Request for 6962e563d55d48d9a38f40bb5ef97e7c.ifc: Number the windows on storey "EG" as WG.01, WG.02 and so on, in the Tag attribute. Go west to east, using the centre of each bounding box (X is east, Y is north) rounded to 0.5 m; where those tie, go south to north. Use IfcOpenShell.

First a look at what the model holds.

```python
import ifcopenshell
import ifcopenshell.util.element
import ifcopenshell.util.placement

model = ifcopenshell.open("6962e563d55d48d9a38f40bb5ef97e7c.ifc")
print(model.schema)
storey = next(s for s in model.by_type("IfcBuildingStorey") if s.Name == "EG")
windows = [e for e in ifcopenshell.util.element.get_decomposition(storey) if e.is_a("IfcWindow")]
for e in sorted(windows, key=lambda e: e.id()):
    origin = ifcopenshell.util.placement.get_local_placement(e.ObjectPlacement)[:3, 3]
    print(e.id(), e.Tag, e.Name, origin.round(2) + 0.0, sep=" | ")
```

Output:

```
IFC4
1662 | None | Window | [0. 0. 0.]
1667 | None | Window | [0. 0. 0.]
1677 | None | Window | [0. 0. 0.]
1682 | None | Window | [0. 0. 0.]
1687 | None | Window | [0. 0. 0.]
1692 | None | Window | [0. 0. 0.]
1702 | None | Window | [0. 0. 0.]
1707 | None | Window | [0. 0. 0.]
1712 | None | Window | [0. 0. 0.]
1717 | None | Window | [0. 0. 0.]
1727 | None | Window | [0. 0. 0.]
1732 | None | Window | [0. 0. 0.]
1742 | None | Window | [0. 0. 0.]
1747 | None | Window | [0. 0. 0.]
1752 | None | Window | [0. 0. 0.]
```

```python
import ifcopenshell
import ifcopenshell.geom
import ifcopenshell.util.element
import ifcopenshell.util.shape

model = ifcopenshell.open("6962e563d55d48d9a38f40bb5ef97e7c.ifc")
settings = ifcopenshell.geom.settings()
settings.set("use-world-coords", True)


def centre(element):
    shape = ifcopenshell.geom.create_shape(settings, element)
    return ifcopenshell.util.shape.get_bbox_centroid(shape.geometry)


storey = next(s for s in model.by_type("IfcBuildingStorey") if s.Name == "EG")
windows = [e for e in ifcopenshell.util.element.get_decomposition(storey) if e.is_a("IfcWindow")]

# Insertion points can sit at a corner or the storey origin, so sort by the geometry (in metres).
centres = {e: centre(e) for e in windows}
windows.sort(key=lambda e: (round(centres[e][0] / 0.5), centres[e][1]))

for i, e in enumerate(windows, start=1):
    number = f"WG.{i:02d}"
    e.Tag = number
    print(e.id(), number)

model.write("6962e563d55d48d9a38f40bb5ef97e7c_rev.ifc")
```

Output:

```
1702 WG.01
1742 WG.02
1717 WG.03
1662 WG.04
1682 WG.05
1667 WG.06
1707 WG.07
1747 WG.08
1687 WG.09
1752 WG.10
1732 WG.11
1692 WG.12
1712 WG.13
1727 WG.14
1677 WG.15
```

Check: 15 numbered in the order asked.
